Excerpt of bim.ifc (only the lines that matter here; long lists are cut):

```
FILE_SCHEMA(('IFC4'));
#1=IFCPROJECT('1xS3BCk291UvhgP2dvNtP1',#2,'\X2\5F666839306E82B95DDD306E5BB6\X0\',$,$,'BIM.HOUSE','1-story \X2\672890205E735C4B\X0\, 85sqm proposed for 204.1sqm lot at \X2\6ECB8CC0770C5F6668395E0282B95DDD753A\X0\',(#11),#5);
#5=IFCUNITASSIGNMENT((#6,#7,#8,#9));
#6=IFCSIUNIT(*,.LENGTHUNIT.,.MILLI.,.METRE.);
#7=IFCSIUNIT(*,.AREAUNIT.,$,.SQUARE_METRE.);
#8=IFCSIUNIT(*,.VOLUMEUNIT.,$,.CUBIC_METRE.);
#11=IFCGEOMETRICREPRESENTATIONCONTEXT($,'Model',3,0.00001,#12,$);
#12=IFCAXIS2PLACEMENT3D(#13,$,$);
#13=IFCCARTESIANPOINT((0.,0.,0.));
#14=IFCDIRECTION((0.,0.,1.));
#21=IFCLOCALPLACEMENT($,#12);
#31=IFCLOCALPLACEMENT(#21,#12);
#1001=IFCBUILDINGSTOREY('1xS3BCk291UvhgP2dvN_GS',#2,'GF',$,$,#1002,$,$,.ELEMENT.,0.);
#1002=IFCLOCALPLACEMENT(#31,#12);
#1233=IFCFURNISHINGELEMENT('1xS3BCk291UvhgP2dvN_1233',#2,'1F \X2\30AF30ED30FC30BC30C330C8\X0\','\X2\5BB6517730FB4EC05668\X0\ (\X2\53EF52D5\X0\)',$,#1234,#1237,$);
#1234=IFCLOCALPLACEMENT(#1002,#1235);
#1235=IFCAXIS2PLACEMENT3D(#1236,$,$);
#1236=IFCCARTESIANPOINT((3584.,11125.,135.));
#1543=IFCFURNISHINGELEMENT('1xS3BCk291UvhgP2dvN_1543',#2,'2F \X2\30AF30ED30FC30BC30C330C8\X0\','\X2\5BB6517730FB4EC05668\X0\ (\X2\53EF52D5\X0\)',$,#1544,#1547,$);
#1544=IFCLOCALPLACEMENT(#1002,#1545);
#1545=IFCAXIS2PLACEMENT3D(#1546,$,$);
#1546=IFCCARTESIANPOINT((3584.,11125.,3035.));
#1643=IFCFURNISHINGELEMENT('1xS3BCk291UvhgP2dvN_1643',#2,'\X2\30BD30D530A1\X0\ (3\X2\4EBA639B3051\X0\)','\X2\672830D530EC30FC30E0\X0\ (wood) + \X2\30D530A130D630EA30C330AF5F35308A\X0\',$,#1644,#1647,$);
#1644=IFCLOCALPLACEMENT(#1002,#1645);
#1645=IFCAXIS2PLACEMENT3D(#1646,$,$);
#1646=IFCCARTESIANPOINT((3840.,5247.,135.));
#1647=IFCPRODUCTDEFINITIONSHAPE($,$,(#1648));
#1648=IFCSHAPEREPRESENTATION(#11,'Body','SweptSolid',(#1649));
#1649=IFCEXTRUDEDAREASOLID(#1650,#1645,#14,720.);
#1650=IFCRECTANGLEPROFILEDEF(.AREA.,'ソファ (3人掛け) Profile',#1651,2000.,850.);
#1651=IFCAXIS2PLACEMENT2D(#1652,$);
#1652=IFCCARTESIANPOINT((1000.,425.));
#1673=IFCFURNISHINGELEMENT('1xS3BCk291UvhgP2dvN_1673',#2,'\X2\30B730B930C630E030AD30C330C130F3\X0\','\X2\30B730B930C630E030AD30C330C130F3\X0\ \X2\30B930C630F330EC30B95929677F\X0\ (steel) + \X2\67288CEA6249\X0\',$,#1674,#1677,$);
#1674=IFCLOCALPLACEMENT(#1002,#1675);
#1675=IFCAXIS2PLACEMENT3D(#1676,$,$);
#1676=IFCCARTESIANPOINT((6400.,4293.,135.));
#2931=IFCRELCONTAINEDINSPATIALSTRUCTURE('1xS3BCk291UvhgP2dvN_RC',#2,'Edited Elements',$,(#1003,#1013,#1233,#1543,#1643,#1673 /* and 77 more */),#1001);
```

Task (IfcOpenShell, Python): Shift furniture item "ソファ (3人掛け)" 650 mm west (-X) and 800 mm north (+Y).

```python
import ifcopenshell
import ifcopenshell.api.geometry
import ifcopenshell.util.placement

model = ifcopenshell.open("bim.ifc")

item = model.by_guid("1xS3BCk291UvhgP2dvN_1643")
matrix = ifcopenshell.util.placement.get_local_placement(item.ObjectPlacement)
matrix[0, 3] -= 650.0
matrix[1, 3] += 800.0
ifcopenshell.api.geometry.edit_object_placement(model, product=item, matrix=matrix, is_si=False)

print(ifcopenshell.util.placement.get_local_placement(item.ObjectPlacement).round(3) + 0.0)

model.write("bim-out.ifc")
```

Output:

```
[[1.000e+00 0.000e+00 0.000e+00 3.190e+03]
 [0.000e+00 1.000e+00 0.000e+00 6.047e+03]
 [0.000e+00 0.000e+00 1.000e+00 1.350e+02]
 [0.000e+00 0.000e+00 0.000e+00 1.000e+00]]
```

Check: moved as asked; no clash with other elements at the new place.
